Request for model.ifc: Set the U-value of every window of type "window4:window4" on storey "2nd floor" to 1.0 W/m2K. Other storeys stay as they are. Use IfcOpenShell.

First a look at what the model holds.

```python
import ifcopenshell
import ifcopenshell.util.element

model = ifcopenshell.open("model.ifc")
print(model.schema)
storey = next(s for s in model.by_type("IfcBuildingStorey") if s.Name == "2nd floor")
windows = [e for e in ifcopenshell.util.element.get_decomposition(storey) if e.is_a("IfcWindow")]
seen = {}
for e in windows:
    element_type = ifcopenshell.util.element.get_type(e)
    key = (element_type.Name if element_type != e and element_type else None, ifcopenshell.util.element.get_pset(e, "Pset_WindowCommon", "ThermalTransmittance"))
    seen[key] = seen.get(key, 0) + 1
for (name, value), count in sorted(seen.items(), key=str):
    print(count, "x", name, "|", value)
```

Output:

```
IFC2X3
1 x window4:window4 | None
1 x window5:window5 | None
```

```python
import ifcopenshell
import ifcopenshell.api.pset
import ifcopenshell.util.element

model = ifcopenshell.open("model.ifc")

storey = next(s for s in model.by_type("IfcBuildingStorey") if s.Name == "2nd floor")
windows = [e for e in ifcopenshell.util.element.get_decomposition(storey) if e.is_a("IfcWindow")]

count = 0
for e in windows:
    element_type = ifcopenshell.util.element.get_type(e)
    if element_type in (None, e) or element_type.Name != "window4:window4":
        continue
    # add_pset returns the element's existing set when there is one.
    pset = ifcopenshell.api.pset.add_pset(model, product=e, name="Pset_WindowCommon")
    ifcopenshell.api.pset.edit_pset(model, pset=pset, properties={"ThermalTransmittance": 1.0})
    count += 1

print(count, "windows updated")

model.write("model_edited.ifc")
```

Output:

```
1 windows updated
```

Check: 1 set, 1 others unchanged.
